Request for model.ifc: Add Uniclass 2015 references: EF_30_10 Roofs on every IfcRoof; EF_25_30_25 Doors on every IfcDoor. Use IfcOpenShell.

First a look at what the model holds.

```python
import ifcopenshell

model = ifcopenshell.open("model.ifc")
print(model.schema)
print("classifications:", [c.Name for c in model.by_type("IfcClassification")])
for ifc_class in ("IfcDoor", "IfcRoof", "IfcStair", "IfcWall", "IfcWindow"):
    print(ifc_class, len(model.by_type(ifc_class)))
```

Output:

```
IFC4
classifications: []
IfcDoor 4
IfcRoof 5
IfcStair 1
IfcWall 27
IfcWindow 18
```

```python
import ifcopenshell
import ifcopenshell.api.classification

model = ifcopenshell.open("model.ifc")

system = ifcopenshell.api.classification.add_classification(model, classification="Uniclass 2015")

codes = {
    "IfcRoof": ("EF_30_10", "Roofs"),
    "IfcDoor": ("EF_25_30_25", "Doors"),
}
for ifc_class, (code, name) in codes.items():
    products = model.by_type(ifc_class)
    ifcopenshell.api.classification.add_reference(
        model, products=products, classification=system, identification=code, name=name
    )
    print(code, len(products))

model.write("model_v2.ifc")
```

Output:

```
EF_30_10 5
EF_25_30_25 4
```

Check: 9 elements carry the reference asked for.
